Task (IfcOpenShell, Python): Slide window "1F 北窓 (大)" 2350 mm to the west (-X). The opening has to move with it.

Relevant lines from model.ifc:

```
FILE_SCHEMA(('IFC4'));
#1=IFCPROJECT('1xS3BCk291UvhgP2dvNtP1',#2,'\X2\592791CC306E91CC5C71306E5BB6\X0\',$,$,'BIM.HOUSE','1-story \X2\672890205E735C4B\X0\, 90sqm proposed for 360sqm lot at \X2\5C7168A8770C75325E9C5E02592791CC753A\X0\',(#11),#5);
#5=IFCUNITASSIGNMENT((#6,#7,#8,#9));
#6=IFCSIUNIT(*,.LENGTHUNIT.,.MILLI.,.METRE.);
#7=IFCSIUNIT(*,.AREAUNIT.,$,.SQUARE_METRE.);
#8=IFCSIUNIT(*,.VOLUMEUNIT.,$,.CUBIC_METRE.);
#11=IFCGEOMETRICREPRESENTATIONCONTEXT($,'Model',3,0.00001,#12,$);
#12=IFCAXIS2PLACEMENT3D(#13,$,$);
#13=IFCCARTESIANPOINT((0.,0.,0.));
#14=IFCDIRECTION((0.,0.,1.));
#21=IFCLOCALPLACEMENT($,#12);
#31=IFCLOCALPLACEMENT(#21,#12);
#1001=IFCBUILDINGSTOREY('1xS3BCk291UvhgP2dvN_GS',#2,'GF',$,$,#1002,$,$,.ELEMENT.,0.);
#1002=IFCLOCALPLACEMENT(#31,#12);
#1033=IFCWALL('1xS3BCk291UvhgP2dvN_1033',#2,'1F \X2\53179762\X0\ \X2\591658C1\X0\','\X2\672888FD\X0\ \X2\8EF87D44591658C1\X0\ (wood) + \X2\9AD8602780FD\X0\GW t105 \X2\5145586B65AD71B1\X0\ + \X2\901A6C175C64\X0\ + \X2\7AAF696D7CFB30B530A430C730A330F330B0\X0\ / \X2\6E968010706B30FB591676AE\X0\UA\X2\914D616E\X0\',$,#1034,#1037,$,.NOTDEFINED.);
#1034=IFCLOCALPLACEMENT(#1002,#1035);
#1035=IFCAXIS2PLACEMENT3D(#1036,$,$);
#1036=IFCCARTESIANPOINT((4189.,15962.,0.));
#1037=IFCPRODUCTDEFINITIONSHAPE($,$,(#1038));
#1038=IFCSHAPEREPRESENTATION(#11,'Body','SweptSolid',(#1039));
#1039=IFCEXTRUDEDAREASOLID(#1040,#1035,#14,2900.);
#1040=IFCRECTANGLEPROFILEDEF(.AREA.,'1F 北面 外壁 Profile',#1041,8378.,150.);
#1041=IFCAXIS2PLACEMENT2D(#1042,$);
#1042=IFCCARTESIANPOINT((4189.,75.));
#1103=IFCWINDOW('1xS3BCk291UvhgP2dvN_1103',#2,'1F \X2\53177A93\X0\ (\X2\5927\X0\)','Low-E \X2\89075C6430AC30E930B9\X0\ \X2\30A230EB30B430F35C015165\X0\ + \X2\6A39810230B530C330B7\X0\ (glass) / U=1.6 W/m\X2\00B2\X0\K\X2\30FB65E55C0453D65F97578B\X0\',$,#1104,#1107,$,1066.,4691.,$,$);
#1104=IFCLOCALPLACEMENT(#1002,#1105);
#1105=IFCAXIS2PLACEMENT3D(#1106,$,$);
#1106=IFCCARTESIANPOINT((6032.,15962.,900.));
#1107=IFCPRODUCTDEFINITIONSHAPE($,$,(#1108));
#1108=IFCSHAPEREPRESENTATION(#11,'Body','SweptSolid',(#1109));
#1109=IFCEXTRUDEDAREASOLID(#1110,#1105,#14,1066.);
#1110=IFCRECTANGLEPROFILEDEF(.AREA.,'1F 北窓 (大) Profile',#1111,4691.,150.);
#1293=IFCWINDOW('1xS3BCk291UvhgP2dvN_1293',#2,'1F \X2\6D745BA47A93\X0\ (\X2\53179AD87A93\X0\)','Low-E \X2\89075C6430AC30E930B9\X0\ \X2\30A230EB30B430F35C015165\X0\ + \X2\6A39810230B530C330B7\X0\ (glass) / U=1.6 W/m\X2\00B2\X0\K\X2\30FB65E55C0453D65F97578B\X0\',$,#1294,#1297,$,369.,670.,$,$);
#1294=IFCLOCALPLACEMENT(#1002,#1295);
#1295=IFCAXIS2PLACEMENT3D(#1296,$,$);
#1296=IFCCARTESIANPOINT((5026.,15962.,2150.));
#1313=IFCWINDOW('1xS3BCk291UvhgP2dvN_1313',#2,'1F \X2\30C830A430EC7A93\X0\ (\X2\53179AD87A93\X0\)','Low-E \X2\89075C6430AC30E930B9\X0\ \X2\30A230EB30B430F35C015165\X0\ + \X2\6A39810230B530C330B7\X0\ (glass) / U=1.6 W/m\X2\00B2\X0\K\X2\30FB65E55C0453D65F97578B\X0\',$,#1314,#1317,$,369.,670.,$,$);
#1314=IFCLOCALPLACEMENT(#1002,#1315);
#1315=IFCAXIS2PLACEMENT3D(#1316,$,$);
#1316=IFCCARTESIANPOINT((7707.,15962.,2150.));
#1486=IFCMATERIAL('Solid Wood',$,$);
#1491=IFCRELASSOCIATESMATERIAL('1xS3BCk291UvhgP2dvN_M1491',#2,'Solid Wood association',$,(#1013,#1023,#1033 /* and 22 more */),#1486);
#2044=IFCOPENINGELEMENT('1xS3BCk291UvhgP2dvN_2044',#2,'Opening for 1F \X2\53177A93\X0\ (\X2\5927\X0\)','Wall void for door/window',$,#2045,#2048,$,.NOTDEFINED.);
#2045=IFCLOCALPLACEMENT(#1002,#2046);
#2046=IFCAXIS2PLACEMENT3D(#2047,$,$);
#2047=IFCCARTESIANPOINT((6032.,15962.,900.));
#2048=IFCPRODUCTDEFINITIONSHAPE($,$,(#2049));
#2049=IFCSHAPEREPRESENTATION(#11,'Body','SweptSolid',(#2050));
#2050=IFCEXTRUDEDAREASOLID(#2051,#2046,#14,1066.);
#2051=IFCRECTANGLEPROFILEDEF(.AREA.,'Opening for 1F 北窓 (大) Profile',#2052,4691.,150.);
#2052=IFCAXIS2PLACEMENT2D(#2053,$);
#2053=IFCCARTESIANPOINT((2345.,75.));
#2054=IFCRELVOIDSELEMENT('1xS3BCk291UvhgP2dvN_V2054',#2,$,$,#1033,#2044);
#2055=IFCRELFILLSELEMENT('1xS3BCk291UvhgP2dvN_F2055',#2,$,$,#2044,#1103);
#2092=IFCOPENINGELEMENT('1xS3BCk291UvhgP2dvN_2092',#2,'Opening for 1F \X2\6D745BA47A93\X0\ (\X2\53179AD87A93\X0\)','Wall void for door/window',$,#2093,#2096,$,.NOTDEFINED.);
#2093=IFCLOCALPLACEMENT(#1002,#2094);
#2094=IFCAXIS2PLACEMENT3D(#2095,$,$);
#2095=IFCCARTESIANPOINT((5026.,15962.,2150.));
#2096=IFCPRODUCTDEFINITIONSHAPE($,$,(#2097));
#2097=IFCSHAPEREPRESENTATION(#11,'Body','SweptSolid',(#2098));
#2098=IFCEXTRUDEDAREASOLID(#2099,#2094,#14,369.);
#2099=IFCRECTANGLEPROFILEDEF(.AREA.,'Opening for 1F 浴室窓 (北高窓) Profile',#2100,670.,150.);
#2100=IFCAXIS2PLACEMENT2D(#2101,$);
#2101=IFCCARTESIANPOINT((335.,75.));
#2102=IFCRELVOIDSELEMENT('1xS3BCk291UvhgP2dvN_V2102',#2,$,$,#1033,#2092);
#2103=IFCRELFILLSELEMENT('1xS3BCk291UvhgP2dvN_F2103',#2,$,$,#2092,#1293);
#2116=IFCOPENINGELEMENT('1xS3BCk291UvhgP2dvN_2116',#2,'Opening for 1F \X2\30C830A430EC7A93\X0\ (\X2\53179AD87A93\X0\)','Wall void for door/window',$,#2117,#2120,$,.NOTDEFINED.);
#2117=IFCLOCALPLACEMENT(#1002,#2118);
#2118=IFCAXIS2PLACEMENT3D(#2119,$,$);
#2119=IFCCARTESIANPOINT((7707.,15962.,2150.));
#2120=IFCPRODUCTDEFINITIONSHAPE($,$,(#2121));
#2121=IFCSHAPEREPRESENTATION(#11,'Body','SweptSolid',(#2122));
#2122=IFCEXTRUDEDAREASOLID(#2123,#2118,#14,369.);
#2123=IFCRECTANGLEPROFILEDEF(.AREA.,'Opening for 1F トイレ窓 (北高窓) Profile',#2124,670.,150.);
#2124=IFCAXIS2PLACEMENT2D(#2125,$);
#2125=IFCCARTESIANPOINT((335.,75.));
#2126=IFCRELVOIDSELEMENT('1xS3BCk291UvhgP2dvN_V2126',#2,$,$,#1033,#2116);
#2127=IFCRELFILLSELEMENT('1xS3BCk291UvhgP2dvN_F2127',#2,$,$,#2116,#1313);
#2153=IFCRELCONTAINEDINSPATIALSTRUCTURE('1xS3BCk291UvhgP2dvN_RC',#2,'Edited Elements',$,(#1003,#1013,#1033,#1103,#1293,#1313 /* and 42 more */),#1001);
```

```python
import ifcopenshell
import ifcopenshell.api.geometry
import ifcopenshell.util.placement
import ifcopenshell.util.unit

model = ifcopenshell.open("model.ifc")
unit_scale = ifcopenshell.util.unit.calculate_unit_scale(model)

window = model.by_guid("1xS3BCk291UvhgP2dvN_1103")
opening = window.FillsVoids[0].RelatingOpeningElement
wall = opening.VoidsElements[0].RelatingBuildingElement

wall_matrix = ifcopenshell.util.placement.get_local_placement(wall.ObjectPlacement)
shift = wall_matrix[:3, 0] * -2.35 / unit_scale
before = ifcopenshell.util.placement.get_local_placement(window.ObjectPlacement)[:3, 3].copy()

# The window is not placed relative to its opening, so move both.
for product in (opening, window):
    matrix = ifcopenshell.util.placement.get_local_placement(product.ObjectPlacement)
    matrix[:3, 3] += shift
    ifcopenshell.api.geometry.edit_object_placement(model, product=product, matrix=matrix, is_si=False)

after = ifcopenshell.util.placement.get_local_placement(window.ObjectPlacement)[:3, 3]
print("window moved by", (after - before).round(3) + 0.0)

model.write("model_edited.ifc")
```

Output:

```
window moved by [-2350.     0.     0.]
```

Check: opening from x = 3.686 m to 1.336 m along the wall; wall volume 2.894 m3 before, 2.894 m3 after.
